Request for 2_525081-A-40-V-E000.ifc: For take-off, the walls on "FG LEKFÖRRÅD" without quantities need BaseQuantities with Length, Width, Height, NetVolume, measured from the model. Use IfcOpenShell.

First a look at what the model holds.

```python
import ifcopenshell
import ifcopenshell.util.element
import ifcopenshell.util.unit

model = ifcopenshell.open("2_525081-A-40-V-E000.ifc")
print(model.schema)
for unit_type in ("LENGTHUNIT", "AREAUNIT", "VOLUMEUNIT"):
    print(unit_type, ifcopenshell.util.unit.calculate_unit_scale(model, unit_type))
storey = next(s for s in model.by_type("IfcBuildingStorey") if s.Name == "FG LEKFÖRRÅD")
walls = [e for e in ifcopenshell.util.element.get_decomposition(storey) if e.is_a("IfcWall")]
for e in sorted(walls, key=lambda e: e.id()):
    print(e.id(), e.is_a(), e.Name, list(ifcopenshell.util.element.get_psets(e, qtos_only=True)), sep=" | ")
```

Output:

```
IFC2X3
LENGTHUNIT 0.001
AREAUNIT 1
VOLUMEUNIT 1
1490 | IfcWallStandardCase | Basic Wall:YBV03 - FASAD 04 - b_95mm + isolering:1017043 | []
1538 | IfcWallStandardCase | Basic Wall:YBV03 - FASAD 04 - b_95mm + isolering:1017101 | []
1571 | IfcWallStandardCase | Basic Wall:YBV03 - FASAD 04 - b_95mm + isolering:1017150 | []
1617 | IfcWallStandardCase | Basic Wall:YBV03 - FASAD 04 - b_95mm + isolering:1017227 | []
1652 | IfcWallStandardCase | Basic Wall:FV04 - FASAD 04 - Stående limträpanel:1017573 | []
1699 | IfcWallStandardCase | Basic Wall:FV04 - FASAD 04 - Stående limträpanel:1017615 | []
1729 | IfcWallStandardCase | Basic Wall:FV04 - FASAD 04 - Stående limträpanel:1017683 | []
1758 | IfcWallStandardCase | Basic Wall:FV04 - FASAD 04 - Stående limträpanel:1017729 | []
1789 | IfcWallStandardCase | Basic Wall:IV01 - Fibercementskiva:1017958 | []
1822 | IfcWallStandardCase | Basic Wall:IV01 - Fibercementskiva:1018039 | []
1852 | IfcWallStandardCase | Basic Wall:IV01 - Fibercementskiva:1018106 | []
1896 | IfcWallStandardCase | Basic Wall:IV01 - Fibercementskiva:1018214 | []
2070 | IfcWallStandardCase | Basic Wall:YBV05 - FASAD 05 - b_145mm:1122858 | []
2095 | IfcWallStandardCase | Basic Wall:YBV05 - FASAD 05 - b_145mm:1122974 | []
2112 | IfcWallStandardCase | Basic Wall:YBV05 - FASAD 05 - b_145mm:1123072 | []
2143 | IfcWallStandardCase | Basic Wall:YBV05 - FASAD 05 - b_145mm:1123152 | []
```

```python
import ifcopenshell
import ifcopenshell.api.pset
import ifcopenshell.geom
import ifcopenshell.util.element
import ifcopenshell.util.shape
import ifcopenshell.util.unit

model = ifcopenshell.open("2_525081-A-40-V-E000.ifc")
unit_scale = ifcopenshell.util.unit.calculate_unit_scale(model)
volume_scale = ifcopenshell.util.unit.calculate_unit_scale(model, "VOLUMEUNIT")
settings = ifcopenshell.geom.settings()

storey = next(s for s in model.by_type("IfcBuildingStorey") if s.Name == "FG LEKFÖRRÅD")
walls = [e for e in ifcopenshell.util.element.get_decomposition(storey) if e.is_a("IfcWall")]

for e in sorted(walls, key=lambda e: e.id()):
    if ifcopenshell.util.element.get_psets(e, qtos_only=True, should_inherit=False):
        continue
    # Geometry comes back in metres, in the element's own axes.
    shape = ifcopenshell.geom.create_shape(settings, e)
    values = {
        "Length": ifcopenshell.util.shape.get_x(shape.geometry) / unit_scale,
        "Width": ifcopenshell.util.shape.get_y(shape.geometry) / unit_scale,
        "Height": ifcopenshell.util.shape.get_z(shape.geometry) / unit_scale,
        "NetVolume": ifcopenshell.util.shape.get_volume(shape.geometry) / volume_scale,
    }
    qto = ifcopenshell.api.pset.add_qto(model, product=e, name="BaseQuantities")
    ifcopenshell.api.pset.edit_qto(model, qto=qto, properties=values)
    print(e.id(), {k: round(v, 3) for k, v in values.items()})

model.write("2_525081-A-40-V-E000_rev.ifc")
```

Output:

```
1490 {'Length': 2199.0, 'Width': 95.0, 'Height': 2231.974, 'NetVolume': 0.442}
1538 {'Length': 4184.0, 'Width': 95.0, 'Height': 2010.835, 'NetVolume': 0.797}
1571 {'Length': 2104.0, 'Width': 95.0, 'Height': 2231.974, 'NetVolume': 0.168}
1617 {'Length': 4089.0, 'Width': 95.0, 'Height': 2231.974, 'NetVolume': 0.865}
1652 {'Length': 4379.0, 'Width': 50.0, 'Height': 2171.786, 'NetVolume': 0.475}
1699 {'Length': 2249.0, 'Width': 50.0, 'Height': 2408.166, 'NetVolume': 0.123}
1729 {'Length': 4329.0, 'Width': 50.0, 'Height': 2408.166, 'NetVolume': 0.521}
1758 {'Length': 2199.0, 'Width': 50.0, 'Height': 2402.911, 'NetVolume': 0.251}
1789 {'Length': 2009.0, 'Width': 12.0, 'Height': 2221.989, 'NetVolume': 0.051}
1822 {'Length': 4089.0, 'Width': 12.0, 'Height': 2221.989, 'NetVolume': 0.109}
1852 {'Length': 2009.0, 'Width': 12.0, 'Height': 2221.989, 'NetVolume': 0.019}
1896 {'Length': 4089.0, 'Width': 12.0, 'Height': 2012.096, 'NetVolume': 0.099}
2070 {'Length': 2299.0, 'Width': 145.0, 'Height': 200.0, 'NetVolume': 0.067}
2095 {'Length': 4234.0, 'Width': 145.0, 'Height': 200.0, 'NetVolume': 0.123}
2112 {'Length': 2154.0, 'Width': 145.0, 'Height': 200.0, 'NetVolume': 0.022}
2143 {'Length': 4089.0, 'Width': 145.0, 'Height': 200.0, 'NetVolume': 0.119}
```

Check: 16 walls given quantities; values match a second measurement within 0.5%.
